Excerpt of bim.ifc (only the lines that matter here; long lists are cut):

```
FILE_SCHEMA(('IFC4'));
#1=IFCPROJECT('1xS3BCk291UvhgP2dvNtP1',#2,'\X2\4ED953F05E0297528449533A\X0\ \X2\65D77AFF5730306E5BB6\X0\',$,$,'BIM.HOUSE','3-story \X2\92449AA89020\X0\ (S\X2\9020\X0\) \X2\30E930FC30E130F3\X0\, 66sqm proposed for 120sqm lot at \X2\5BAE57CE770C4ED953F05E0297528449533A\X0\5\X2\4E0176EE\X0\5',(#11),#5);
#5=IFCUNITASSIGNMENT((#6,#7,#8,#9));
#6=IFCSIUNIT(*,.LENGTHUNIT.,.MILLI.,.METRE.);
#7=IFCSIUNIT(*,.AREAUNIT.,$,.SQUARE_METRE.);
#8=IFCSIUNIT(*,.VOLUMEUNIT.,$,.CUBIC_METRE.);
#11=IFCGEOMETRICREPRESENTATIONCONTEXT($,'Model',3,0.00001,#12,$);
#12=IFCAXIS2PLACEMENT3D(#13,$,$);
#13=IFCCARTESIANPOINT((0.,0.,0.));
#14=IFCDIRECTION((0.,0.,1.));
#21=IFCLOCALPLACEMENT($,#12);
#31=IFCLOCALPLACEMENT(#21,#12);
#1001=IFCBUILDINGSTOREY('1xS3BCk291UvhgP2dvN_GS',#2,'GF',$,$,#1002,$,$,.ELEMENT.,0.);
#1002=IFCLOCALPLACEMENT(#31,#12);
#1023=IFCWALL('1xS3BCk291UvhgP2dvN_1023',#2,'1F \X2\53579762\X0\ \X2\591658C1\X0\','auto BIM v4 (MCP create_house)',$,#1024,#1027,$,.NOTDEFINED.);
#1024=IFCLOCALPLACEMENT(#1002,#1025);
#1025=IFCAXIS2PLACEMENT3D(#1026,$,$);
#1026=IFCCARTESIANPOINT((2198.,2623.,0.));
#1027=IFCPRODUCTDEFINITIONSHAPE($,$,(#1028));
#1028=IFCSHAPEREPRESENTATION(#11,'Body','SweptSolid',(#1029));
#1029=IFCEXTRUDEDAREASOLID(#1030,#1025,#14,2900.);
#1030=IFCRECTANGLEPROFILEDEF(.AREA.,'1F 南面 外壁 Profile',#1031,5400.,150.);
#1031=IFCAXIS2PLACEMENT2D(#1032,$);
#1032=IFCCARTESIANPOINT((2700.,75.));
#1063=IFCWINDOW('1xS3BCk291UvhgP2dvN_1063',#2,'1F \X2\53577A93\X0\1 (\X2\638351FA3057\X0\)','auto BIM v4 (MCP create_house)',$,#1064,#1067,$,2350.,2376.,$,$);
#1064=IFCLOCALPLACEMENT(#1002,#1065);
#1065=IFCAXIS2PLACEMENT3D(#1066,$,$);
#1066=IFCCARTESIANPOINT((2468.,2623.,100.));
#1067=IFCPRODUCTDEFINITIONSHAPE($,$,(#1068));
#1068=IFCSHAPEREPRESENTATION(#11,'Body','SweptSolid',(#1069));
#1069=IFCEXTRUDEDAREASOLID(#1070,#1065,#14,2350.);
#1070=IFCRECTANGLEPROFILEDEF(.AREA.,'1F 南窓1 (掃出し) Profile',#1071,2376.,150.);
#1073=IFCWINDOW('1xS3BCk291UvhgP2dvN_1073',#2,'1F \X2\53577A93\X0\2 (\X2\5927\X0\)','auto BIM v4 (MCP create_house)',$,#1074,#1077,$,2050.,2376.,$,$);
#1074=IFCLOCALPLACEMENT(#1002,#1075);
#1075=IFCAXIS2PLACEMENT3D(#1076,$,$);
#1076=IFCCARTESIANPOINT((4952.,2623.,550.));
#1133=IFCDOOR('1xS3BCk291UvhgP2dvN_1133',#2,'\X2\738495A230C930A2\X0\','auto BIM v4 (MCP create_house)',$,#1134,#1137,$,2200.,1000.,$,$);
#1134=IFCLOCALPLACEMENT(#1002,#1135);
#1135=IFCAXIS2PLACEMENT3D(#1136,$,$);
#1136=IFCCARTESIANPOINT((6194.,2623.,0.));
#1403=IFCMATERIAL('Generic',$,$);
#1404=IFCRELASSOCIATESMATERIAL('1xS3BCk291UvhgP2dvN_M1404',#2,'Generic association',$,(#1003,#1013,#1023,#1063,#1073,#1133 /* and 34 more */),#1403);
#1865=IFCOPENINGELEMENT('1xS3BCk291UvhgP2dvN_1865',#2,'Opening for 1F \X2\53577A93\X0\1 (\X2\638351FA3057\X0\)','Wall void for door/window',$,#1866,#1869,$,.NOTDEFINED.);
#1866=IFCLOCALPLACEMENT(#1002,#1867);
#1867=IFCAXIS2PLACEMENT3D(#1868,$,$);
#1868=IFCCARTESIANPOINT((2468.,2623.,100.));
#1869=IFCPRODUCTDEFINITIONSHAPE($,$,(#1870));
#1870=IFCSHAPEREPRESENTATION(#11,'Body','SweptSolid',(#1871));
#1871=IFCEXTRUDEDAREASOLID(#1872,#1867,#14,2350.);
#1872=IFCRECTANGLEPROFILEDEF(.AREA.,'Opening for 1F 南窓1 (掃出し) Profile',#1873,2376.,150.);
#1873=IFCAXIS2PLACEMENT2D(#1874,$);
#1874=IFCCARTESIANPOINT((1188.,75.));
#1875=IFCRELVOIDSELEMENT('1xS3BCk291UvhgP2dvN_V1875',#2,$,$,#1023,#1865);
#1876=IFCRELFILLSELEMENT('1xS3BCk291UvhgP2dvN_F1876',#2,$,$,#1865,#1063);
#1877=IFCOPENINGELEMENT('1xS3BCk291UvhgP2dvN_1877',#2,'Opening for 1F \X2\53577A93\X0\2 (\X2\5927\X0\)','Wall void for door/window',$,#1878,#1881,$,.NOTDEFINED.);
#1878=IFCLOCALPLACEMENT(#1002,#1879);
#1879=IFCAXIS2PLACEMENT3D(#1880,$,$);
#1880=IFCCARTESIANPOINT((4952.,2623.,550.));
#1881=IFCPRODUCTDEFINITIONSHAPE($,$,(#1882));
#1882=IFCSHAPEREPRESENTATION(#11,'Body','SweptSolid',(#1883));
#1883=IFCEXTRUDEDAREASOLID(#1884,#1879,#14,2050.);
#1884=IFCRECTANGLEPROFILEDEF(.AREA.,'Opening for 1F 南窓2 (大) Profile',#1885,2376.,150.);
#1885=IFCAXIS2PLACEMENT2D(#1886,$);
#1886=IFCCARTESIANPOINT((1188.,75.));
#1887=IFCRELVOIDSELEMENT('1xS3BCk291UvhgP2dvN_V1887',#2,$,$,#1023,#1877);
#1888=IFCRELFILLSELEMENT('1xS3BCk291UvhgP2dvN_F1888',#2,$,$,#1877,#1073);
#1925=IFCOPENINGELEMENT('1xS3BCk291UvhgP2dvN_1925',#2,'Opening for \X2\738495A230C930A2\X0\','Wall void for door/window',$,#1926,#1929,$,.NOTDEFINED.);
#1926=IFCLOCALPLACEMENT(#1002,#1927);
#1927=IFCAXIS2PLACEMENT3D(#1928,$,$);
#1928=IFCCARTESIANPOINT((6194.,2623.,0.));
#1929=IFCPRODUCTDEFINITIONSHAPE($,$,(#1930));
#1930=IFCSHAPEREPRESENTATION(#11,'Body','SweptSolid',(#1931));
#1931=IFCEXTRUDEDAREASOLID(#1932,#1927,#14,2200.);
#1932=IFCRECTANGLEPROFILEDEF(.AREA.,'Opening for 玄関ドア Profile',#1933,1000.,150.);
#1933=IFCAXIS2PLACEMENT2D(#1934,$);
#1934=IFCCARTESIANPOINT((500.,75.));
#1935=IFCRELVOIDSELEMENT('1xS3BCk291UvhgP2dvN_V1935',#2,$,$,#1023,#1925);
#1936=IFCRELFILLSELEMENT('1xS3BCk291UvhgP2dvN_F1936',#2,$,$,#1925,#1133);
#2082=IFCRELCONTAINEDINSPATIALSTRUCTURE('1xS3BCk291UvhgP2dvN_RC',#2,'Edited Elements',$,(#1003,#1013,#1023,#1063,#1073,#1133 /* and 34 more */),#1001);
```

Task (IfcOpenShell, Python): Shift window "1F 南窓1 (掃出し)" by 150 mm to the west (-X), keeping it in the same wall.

```python
import ifcopenshell
import ifcopenshell.api.geometry
import ifcopenshell.util.placement

model = ifcopenshell.open("bim.ifc")

window = model.by_guid("1xS3BCk291UvhgP2dvN_1063")
opening = window.FillsVoids[0].RelatingOpeningElement
wall = opening.VoidsElements[0].RelatingBuildingElement

wall_matrix = ifcopenshell.util.placement.get_local_placement(wall.ObjectPlacement)
shift = wall_matrix[:3, 0] * -150.0
before = ifcopenshell.util.placement.get_local_placement(window.ObjectPlacement)[:3, 3].copy()

# The window is not placed relative to its opening, so move both.
for product in (opening, window):
    matrix = ifcopenshell.util.placement.get_local_placement(product.ObjectPlacement)
    matrix[:3, 3] += shift
    ifcopenshell.api.geometry.edit_object_placement(model, product=product, matrix=matrix, is_si=False)

after = ifcopenshell.util.placement.get_local_placement(window.ObjectPlacement)[:3, 3]
print("window moved by", (after - before).round(3) + 0.0)

model.write("bim-out.ifc")
```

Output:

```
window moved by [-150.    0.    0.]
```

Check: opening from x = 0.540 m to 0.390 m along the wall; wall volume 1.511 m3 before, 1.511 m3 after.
